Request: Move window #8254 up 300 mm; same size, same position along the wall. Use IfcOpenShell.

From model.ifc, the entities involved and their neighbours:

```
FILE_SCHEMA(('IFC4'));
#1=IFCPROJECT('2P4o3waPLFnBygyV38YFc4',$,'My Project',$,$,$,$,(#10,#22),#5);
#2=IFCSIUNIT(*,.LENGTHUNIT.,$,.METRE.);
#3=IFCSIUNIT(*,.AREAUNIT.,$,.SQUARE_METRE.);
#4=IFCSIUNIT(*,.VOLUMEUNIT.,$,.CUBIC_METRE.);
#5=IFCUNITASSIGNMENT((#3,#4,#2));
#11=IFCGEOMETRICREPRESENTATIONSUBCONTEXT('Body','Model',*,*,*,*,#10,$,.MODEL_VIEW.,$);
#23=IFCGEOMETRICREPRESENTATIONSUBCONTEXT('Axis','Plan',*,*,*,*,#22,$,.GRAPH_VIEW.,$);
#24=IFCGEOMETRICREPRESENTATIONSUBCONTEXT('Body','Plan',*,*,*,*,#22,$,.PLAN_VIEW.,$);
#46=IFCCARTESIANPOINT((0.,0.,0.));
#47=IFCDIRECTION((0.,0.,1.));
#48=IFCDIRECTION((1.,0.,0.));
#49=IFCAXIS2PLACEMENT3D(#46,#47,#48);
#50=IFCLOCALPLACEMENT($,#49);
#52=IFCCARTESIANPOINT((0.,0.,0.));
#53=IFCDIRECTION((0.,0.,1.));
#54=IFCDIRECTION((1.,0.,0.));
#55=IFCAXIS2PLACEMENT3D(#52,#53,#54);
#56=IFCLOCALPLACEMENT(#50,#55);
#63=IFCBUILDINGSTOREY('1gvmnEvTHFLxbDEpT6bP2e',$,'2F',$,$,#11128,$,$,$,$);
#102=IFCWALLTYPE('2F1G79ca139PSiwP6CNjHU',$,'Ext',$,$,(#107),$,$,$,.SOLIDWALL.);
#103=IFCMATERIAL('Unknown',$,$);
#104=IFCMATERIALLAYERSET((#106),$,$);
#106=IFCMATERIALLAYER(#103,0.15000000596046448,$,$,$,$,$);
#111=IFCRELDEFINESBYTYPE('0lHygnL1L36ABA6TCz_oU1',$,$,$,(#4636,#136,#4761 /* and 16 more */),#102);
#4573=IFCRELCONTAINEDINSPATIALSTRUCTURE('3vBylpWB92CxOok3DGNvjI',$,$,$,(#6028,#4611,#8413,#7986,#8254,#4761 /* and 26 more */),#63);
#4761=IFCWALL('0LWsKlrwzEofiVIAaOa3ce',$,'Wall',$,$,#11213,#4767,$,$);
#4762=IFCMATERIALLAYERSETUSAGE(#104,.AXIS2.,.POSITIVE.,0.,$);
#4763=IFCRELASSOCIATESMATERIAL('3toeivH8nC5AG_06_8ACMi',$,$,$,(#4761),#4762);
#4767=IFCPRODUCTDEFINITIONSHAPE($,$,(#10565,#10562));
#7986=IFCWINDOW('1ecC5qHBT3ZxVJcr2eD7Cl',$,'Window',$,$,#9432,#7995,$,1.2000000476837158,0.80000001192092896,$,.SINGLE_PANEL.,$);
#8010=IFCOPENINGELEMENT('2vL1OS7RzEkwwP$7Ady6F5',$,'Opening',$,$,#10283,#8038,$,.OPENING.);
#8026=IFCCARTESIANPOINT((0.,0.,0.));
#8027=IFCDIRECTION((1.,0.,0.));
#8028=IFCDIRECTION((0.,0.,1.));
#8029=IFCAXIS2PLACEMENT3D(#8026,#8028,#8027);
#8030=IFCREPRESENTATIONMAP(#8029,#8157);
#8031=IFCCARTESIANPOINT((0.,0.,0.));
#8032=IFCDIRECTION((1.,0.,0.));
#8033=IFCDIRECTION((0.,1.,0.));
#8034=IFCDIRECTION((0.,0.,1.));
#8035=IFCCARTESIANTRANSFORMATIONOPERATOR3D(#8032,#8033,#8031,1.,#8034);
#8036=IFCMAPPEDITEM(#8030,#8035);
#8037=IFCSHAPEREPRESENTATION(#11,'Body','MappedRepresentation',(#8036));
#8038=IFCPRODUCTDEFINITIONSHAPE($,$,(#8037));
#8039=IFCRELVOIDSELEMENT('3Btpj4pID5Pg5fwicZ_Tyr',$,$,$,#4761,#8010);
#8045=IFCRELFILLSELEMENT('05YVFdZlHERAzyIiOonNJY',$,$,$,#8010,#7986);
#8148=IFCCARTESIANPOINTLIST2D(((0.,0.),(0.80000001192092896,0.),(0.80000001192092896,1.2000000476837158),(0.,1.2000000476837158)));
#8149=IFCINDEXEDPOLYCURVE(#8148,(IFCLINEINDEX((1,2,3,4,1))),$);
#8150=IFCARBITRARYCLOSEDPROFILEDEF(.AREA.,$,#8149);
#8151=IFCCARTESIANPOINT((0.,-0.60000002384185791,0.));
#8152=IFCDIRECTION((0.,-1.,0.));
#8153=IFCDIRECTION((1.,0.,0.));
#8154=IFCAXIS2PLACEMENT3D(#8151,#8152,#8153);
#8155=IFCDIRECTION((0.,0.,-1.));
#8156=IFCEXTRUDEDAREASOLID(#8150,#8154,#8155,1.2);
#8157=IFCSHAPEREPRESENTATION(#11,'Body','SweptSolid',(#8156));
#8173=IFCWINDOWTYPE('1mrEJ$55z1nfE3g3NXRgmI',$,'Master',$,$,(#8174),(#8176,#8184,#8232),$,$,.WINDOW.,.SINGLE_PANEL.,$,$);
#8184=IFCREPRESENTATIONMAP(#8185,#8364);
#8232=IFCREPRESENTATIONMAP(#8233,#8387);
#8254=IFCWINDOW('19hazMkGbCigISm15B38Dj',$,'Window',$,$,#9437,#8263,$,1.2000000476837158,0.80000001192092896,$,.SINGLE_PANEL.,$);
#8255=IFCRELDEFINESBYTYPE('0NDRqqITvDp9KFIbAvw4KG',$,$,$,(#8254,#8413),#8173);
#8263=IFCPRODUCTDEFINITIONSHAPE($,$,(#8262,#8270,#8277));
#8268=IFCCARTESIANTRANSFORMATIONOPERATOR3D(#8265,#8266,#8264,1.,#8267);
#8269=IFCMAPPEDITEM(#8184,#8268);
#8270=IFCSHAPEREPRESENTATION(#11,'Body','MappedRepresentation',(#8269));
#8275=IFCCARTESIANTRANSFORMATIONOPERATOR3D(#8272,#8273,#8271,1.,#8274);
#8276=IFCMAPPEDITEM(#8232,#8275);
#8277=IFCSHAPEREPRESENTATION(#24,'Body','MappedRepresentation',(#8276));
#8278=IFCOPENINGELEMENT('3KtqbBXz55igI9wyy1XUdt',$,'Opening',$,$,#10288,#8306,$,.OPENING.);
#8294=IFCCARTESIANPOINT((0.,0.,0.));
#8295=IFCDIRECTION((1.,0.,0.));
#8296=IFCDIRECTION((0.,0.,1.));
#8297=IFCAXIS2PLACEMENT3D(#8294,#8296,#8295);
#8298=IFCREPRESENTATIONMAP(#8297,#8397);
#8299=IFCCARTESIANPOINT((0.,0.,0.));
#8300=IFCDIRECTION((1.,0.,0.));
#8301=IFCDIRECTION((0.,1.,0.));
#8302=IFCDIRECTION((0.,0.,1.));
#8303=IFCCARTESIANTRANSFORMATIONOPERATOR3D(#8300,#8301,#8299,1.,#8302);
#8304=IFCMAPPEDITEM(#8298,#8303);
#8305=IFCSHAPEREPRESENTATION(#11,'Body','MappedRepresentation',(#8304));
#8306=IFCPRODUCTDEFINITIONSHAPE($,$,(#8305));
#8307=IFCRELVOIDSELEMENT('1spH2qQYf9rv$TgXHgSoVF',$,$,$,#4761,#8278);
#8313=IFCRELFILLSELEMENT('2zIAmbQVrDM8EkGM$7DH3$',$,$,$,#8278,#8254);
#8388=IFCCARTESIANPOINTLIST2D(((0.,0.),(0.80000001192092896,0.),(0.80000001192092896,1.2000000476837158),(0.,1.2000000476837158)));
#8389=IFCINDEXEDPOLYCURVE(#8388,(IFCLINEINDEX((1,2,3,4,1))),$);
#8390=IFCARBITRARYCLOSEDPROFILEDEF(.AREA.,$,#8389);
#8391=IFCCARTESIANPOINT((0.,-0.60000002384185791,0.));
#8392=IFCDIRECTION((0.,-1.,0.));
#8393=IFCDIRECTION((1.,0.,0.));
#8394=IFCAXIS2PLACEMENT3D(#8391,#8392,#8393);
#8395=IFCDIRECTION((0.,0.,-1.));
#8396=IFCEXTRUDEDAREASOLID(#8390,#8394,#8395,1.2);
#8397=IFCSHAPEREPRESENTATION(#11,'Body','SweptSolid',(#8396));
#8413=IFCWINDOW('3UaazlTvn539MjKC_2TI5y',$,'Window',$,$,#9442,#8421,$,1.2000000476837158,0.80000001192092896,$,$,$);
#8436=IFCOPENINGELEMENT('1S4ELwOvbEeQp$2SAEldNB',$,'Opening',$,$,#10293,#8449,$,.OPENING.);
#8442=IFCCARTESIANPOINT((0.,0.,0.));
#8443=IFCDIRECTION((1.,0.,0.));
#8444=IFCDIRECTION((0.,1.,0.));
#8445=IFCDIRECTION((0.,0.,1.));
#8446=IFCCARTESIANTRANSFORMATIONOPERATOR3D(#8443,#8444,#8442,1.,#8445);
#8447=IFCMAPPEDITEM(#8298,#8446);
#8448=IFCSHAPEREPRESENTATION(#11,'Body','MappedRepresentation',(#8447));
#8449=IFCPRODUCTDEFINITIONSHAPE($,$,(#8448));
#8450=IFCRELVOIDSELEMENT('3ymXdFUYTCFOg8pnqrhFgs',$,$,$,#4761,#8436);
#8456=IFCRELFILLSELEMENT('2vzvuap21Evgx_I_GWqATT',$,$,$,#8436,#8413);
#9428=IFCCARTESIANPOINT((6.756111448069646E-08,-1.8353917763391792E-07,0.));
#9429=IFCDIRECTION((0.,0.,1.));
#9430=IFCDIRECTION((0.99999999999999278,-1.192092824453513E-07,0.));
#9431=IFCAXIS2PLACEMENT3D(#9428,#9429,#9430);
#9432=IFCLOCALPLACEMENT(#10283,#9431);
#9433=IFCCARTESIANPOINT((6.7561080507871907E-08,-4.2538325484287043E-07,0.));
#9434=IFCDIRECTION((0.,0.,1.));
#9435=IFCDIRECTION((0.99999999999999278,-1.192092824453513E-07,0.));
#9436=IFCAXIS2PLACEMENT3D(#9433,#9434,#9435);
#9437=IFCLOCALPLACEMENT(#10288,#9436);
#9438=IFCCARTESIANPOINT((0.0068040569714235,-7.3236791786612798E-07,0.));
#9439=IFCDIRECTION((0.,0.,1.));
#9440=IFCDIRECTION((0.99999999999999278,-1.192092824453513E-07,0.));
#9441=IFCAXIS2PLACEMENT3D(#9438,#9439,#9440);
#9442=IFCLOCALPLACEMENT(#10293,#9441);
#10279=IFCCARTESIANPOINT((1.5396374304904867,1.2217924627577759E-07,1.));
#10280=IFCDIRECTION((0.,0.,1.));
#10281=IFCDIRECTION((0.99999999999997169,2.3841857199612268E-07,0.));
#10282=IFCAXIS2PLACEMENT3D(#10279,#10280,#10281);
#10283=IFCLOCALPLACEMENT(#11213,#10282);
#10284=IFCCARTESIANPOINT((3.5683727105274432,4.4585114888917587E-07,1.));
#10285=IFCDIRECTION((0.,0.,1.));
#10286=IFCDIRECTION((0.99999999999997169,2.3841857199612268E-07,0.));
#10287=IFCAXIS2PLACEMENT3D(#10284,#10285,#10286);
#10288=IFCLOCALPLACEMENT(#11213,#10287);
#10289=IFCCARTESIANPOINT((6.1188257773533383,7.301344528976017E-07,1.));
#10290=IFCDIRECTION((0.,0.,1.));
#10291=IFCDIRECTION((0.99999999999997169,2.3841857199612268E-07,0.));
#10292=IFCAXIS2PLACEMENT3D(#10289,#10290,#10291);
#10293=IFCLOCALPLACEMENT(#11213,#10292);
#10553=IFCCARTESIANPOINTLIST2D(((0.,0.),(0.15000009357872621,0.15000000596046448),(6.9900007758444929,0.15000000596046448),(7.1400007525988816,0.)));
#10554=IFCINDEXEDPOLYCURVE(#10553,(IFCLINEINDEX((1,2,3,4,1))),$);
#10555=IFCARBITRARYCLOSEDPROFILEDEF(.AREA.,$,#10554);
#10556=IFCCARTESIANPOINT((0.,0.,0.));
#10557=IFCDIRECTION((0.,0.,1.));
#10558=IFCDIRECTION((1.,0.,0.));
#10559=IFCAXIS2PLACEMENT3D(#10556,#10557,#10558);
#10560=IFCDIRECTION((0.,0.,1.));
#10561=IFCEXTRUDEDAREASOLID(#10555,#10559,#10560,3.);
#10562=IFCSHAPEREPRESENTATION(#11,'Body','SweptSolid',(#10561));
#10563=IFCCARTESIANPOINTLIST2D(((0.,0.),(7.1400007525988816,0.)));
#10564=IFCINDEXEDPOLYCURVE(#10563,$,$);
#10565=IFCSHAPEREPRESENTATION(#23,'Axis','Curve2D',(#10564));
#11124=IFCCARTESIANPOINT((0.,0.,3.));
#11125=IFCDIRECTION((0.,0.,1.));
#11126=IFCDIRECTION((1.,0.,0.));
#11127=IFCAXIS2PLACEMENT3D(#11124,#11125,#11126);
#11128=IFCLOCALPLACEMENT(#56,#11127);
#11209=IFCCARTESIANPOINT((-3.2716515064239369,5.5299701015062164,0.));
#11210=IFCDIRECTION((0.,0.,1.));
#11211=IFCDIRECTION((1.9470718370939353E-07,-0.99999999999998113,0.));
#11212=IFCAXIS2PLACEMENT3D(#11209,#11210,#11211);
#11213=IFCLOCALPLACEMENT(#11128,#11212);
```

```python
import numpy as np
import ifcopenshell
import ifcopenshell.api.geometry
import ifcopenshell.util.placement
import ifcopenshell.util.unit

model = ifcopenshell.open("model.ifc")
unit_scale = ifcopenshell.util.unit.calculate_unit_scale(model)

window = model.by_guid("19hazMkGbCigISm15B38Dj")
opening = window.FillsVoids[0].RelatingOpeningElement
dz = 0.3 / unit_scale

shift = np.array([0.0, 0.0, dz])
# The window is placed relative to its opening, so it follows when the opening moves.
matrix = ifcopenshell.util.placement.get_local_placement(opening.ObjectPlacement)
matrix[:3, 3] += shift
ifcopenshell.api.geometry.edit_object_placement(
    model, product=opening, matrix=matrix, is_si=False, should_transform_children=True
)

print(f"moved by {dz * unit_scale:+.3f} m")

model.write("model_v2.ifc")
```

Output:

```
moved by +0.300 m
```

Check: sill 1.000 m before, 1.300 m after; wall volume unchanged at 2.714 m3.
